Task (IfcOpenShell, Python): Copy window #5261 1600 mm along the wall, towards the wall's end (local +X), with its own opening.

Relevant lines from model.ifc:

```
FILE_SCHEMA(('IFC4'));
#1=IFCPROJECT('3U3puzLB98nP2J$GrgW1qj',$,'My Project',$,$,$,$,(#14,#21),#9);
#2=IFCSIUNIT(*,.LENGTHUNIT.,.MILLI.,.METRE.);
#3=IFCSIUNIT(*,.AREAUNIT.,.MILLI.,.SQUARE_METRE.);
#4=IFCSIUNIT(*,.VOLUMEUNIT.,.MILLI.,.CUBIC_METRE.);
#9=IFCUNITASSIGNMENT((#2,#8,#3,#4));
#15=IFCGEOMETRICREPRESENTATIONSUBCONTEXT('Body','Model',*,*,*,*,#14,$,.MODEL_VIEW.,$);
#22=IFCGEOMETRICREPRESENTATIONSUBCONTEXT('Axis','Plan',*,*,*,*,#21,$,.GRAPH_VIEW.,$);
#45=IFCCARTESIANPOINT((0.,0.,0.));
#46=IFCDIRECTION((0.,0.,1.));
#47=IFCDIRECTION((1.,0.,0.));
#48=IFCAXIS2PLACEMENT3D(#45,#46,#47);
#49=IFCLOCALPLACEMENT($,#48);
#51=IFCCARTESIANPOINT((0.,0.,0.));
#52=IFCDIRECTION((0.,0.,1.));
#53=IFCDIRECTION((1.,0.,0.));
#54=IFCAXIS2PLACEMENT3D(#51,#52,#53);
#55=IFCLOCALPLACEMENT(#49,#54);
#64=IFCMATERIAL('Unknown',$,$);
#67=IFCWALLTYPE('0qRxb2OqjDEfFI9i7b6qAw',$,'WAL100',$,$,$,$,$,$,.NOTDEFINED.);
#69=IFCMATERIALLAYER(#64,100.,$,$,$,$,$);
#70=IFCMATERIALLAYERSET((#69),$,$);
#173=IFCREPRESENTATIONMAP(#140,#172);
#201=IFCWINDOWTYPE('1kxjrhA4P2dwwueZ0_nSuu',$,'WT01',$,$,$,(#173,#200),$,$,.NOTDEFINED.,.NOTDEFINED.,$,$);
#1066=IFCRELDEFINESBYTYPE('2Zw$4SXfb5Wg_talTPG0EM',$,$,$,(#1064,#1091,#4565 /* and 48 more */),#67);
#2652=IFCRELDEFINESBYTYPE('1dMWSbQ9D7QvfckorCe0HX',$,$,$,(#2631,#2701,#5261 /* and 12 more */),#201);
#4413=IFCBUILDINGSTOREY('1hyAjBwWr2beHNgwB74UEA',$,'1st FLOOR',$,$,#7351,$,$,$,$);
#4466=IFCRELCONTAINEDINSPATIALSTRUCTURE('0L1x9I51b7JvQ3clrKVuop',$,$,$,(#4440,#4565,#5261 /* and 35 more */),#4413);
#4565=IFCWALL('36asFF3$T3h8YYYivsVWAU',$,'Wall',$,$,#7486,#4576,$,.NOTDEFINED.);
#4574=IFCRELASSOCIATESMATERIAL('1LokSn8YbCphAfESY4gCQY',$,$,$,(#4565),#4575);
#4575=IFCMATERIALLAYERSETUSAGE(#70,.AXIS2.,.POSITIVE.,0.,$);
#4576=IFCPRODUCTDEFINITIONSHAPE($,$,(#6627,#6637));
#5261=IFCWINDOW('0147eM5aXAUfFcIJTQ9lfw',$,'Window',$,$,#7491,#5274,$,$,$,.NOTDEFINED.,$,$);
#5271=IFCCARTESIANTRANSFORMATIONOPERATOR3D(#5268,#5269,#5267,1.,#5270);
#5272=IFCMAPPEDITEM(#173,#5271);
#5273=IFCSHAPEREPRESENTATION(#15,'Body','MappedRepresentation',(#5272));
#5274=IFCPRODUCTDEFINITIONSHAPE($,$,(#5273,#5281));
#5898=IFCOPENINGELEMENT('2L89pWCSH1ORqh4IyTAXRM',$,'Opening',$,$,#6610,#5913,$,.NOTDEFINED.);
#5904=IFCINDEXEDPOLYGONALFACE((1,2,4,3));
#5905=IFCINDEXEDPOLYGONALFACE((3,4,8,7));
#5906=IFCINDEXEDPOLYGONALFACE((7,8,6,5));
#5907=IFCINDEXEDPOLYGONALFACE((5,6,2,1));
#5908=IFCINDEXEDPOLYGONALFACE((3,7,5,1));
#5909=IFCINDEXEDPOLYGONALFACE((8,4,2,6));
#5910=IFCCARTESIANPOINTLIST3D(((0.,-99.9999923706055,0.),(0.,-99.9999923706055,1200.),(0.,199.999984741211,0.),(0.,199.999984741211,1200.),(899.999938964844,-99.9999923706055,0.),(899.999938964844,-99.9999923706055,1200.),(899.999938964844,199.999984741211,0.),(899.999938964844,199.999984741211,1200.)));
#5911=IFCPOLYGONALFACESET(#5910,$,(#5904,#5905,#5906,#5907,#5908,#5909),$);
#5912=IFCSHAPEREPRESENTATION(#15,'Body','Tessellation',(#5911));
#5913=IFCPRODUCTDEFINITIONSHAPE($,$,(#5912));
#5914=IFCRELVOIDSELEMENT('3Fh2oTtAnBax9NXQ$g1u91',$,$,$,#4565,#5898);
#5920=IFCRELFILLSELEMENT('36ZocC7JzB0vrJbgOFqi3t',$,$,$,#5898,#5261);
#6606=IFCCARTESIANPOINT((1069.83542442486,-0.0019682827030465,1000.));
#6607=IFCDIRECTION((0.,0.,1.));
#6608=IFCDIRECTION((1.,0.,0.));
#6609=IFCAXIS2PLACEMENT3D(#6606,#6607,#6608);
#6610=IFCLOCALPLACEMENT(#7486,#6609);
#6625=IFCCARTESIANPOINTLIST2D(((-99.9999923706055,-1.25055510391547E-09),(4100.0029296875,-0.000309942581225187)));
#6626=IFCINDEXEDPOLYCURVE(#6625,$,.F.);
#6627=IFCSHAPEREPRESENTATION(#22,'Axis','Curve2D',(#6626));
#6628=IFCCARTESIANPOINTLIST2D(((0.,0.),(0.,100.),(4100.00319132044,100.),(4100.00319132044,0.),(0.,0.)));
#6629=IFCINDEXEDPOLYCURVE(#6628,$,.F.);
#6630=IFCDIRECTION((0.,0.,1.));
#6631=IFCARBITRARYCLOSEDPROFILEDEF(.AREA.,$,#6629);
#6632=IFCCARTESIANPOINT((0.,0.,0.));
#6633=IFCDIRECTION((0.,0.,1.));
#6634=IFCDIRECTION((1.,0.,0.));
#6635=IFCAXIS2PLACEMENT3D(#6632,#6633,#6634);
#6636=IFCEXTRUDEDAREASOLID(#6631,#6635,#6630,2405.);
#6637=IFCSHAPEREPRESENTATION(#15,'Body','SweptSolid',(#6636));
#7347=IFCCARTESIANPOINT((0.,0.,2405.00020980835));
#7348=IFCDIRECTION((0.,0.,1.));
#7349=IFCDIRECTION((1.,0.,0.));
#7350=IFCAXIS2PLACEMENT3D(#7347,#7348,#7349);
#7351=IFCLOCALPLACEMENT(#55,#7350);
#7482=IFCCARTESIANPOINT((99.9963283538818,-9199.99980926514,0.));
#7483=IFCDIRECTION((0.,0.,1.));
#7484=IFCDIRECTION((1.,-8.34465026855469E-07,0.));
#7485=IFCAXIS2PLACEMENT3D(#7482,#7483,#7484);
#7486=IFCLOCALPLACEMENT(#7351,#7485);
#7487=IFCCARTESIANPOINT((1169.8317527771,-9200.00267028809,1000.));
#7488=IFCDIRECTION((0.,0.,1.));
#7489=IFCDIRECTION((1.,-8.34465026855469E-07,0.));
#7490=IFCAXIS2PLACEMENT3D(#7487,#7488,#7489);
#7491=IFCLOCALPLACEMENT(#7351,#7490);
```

```python
import ifcopenshell
import ifcopenshell.api.feature
import ifcopenshell.api.geometry
import ifcopenshell.api.root
import ifcopenshell.geom
import ifcopenshell.util.element
import ifcopenshell.util.placement
import ifcopenshell.util.shape
import ifcopenshell.util.unit

model = ifcopenshell.open("model.ifc")
unit_scale = ifcopenshell.util.unit.calculate_unit_scale(model)
settings = ifcopenshell.geom.settings()


def volume(element):
    """Net volume in cubic metres, openings subtracted."""
    shape = ifcopenshell.geom.create_shape(settings, element)
    return ifcopenshell.util.shape.get_volume(shape.geometry)


window = model.by_guid("0147eM5aXAUfFcIJTQ9lfw")
opening = window.FillsVoids[0].RelatingOpeningElement
wall = opening.VoidsElements[0].RelatingBuildingElement
before = volume(wall)
shift = ifcopenshell.util.placement.get_local_placement(wall.ObjectPlacement)[:3, 0] * 1.6 / unit_scale

# copy_class copies the void relationship, type, container and properties, but no geometry.
new_opening = ifcopenshell.api.root.copy_class(model, product=opening)
new_opening.Representation = ifcopenshell.util.element.copy_deep(
    model, opening.Representation, exclude=["IfcGeometricRepresentationContext", "IfcRepresentationMap"]
)
new_window = ifcopenshell.api.root.copy_class(model, product=window)
new_window.Representation = ifcopenshell.util.element.copy_deep(
    model, window.Representation, exclude=["IfcGeometricRepresentationContext", "IfcRepresentationMap"]
)
ifcopenshell.api.feature.add_filling(model, opening=new_opening, element=new_window)

for old, new in ((opening, new_opening), (window, new_window)):
    matrix = ifcopenshell.util.placement.get_local_placement(old.ObjectPlacement)
    matrix[:3, 3] += shift
    ifcopenshell.api.geometry.edit_object_placement(model, product=new, matrix=matrix, is_si=False)

after = volume(wall)

print(f"wall volume {before:.3f} -> {after:.3f} m3")

model.write("model-out.ifc")
```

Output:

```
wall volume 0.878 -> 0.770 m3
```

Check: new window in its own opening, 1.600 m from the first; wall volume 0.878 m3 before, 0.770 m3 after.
